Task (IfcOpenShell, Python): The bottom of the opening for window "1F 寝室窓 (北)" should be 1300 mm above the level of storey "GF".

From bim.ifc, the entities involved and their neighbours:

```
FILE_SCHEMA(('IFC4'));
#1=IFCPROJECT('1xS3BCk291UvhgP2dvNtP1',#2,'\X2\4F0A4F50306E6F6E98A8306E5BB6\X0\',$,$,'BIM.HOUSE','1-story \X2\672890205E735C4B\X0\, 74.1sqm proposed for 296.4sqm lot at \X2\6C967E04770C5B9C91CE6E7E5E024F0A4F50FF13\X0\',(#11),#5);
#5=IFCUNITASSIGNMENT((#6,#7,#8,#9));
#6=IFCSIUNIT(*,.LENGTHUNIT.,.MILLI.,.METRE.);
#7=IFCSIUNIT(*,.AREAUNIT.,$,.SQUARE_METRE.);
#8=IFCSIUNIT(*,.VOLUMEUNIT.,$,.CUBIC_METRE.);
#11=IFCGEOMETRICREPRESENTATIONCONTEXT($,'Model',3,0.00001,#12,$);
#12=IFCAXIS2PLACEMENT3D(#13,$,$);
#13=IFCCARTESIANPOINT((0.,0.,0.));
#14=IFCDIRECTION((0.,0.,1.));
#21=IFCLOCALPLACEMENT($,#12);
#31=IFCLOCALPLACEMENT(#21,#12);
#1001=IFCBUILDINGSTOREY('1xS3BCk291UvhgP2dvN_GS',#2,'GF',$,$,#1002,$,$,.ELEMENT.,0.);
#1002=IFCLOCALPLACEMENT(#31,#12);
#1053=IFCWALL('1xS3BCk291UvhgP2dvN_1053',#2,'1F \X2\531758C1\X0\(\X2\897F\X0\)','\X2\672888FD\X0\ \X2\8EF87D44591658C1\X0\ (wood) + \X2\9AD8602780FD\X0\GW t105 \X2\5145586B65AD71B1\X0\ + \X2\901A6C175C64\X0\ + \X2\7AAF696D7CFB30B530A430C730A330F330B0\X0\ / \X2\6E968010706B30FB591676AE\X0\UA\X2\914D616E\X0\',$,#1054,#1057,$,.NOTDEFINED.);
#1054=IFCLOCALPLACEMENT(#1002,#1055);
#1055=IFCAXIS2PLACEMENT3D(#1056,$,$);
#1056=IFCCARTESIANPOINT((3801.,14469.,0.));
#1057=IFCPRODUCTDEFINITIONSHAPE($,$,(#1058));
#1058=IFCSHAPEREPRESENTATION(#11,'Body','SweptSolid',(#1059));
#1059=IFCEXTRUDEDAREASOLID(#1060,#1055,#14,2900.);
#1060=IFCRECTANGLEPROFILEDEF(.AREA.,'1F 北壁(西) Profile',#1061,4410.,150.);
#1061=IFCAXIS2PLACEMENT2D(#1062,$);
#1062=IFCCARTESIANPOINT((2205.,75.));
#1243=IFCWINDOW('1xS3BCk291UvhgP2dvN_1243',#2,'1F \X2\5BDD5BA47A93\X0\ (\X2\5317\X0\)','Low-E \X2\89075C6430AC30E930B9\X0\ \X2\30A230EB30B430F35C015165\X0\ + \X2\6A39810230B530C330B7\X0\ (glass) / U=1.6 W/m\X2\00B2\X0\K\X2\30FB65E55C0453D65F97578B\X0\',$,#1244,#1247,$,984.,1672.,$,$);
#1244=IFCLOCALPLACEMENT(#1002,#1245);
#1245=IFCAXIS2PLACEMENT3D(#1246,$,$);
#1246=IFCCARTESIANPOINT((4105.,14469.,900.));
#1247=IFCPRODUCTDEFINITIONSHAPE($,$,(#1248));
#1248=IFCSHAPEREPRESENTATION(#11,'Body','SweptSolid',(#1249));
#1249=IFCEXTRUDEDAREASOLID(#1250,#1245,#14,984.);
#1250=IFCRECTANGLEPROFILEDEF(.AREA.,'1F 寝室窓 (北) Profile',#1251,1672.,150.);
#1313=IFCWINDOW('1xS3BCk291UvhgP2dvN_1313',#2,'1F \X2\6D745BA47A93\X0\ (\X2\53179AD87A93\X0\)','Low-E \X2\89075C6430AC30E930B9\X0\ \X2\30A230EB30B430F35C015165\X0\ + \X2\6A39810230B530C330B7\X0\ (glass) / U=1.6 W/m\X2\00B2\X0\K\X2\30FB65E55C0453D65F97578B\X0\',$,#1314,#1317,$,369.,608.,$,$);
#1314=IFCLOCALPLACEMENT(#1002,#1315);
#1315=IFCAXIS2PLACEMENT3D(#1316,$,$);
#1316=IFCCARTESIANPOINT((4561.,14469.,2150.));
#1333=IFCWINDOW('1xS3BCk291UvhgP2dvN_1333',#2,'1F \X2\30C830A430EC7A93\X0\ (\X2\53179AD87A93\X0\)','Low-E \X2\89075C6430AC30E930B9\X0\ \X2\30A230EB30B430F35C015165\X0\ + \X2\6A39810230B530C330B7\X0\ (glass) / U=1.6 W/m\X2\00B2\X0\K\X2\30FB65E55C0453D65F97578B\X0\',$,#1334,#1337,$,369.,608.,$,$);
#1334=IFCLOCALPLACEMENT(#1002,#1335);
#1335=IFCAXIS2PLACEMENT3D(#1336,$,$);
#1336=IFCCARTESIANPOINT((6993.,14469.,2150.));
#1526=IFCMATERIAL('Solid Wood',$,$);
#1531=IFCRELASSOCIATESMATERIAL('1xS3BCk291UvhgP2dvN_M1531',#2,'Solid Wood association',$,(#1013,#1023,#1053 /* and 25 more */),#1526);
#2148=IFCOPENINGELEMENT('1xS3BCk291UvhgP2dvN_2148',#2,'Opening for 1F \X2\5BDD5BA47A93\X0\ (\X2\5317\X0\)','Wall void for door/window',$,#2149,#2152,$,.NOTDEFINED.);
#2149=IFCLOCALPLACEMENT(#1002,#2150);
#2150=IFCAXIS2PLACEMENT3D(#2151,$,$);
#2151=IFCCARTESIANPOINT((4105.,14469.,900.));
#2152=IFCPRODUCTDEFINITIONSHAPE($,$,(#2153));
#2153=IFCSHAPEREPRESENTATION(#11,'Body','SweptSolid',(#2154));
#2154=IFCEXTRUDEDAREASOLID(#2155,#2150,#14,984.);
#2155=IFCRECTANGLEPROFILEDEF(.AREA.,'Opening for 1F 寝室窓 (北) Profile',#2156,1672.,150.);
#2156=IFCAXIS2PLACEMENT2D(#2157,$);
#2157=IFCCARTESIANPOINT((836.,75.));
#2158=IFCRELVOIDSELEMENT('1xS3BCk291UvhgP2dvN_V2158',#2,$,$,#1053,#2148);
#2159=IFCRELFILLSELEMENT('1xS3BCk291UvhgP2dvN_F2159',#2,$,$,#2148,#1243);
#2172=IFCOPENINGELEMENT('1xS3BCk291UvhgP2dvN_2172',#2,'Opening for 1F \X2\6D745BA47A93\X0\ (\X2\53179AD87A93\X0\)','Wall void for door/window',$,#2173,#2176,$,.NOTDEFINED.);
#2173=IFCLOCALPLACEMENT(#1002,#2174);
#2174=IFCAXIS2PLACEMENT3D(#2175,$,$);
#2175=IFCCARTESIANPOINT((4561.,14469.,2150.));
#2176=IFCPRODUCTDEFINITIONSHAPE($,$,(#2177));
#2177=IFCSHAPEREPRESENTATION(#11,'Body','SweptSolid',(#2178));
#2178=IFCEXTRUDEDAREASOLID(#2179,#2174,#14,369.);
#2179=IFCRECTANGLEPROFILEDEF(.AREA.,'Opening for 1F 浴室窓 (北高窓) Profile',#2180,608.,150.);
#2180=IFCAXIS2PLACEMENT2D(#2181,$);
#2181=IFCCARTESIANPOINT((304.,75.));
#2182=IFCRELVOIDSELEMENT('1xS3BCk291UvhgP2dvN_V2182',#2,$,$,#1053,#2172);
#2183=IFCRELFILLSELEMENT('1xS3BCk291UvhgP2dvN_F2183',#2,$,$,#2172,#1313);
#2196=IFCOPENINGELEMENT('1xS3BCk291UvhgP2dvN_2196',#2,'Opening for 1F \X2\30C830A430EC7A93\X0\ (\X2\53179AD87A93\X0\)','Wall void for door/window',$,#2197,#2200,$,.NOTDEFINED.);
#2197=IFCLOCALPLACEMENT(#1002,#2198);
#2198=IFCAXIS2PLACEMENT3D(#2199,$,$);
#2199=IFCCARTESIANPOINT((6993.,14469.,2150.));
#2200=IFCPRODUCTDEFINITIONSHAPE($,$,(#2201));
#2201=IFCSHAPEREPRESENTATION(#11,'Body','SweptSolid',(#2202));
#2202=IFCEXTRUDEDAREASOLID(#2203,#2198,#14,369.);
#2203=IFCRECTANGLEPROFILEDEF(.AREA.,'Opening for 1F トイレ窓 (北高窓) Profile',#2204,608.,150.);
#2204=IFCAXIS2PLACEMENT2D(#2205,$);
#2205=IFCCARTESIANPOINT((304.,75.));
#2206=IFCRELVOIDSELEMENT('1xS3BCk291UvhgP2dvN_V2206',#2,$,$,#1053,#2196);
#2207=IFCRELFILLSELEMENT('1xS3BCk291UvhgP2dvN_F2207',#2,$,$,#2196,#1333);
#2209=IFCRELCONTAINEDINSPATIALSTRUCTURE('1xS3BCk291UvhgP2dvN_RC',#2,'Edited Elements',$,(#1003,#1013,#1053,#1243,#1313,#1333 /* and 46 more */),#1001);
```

```python
import numpy as np
import ifcopenshell
import ifcopenshell.api.geometry
import ifcopenshell.geom
import ifcopenshell.util.element
import ifcopenshell.util.placement
import ifcopenshell.util.shape
import ifcopenshell.util.unit

model = ifcopenshell.open("bim.ifc")
unit_scale = ifcopenshell.util.unit.calculate_unit_scale(model)

window = model.by_guid("1xS3BCk291UvhgP2dvN_1243")
opening = window.FillsVoids[0].RelatingOpeningElement
storey = ifcopenshell.util.element.get_container(window, ifc_class="IfcBuildingStorey")
level = ifcopenshell.util.placement.get_local_placement(storey.ObjectPlacement)[2, 3]

# The opening's origin need not be at the sill, so measure its lowest point.
shape = ifcopenshell.geom.create_shape(ifcopenshell.geom.settings(), opening)
bottom = ifcopenshell.util.shape.get_shape_bottom_elevation(shape, shape.geometry) / unit_scale
dz = level + 1.3 / unit_scale - bottom

shift = np.array([0.0, 0.0, dz])
# The window is not placed relative to its opening, so move both.
for product in (opening, window):
    matrix = ifcopenshell.util.placement.get_local_placement(product.ObjectPlacement)
    matrix[:3, 3] += shift
    ifcopenshell.api.geometry.edit_object_placement(model, product=product, matrix=matrix, is_si=False)

print(f"moved by {dz * unit_scale:+.3f} m")

model.write("bim_v2.ifc")
```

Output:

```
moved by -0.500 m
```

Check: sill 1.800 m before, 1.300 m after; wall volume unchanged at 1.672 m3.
